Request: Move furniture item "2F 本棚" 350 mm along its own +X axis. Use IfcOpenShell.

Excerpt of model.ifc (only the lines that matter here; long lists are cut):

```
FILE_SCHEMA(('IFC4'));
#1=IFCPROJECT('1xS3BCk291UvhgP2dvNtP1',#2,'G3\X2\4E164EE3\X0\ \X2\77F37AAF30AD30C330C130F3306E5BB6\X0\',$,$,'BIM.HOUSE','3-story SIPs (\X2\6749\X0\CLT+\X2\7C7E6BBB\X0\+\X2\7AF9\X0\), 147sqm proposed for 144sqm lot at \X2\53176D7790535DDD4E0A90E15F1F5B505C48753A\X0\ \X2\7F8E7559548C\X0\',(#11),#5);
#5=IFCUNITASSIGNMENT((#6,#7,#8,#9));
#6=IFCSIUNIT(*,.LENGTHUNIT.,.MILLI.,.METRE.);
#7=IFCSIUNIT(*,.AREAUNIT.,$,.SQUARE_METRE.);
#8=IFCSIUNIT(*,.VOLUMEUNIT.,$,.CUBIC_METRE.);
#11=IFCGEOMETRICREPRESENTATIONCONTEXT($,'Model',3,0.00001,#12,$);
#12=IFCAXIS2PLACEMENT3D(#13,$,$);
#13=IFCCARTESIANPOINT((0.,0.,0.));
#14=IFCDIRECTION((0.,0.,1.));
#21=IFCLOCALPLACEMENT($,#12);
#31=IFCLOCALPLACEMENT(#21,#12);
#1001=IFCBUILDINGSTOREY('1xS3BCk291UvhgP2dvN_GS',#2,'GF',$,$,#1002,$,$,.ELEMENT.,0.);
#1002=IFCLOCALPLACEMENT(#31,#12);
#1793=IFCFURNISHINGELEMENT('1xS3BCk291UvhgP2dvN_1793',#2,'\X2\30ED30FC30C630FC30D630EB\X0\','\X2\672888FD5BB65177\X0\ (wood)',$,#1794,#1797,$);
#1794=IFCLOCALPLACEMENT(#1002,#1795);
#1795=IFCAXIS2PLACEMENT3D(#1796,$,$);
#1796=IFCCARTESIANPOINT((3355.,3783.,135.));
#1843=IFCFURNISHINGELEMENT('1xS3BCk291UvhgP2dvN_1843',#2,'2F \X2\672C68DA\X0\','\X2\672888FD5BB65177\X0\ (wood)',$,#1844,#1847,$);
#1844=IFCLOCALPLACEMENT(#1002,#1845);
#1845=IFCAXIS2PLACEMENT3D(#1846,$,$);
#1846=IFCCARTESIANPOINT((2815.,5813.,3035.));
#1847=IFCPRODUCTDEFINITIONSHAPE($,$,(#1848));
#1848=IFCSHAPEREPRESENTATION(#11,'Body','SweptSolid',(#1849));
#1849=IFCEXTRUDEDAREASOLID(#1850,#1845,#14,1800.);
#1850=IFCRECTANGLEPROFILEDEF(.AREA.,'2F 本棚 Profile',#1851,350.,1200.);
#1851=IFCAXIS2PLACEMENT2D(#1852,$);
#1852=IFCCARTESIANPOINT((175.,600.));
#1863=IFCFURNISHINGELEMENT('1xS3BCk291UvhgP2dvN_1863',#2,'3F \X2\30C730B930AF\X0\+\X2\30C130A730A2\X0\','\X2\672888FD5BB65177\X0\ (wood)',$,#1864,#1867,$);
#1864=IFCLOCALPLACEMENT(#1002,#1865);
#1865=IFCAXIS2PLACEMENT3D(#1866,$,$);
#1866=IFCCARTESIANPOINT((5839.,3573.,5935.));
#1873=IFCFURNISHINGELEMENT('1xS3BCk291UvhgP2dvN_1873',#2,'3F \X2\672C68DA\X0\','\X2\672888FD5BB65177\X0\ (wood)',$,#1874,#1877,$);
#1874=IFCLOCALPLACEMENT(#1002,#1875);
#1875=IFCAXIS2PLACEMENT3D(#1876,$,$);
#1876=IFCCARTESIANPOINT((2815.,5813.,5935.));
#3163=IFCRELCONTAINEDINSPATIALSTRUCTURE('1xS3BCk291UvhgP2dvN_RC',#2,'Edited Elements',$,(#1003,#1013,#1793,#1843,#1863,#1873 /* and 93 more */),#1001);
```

```python
import ifcopenshell
import ifcopenshell.api.geometry
import ifcopenshell.util.placement

model = ifcopenshell.open("model.ifc")

item = model.by_guid("1xS3BCk291UvhgP2dvN_1843")
matrix = ifcopenshell.util.placement.get_local_placement(item.ObjectPlacement)
matrix[:3, 3] += matrix[:3, 0] * 350.0
ifcopenshell.api.geometry.edit_object_placement(model, product=item, matrix=matrix, is_si=False)

print(ifcopenshell.util.placement.get_local_placement(item.ObjectPlacement).round(3) + 0.0)

model.write("model_updated.ifc")
```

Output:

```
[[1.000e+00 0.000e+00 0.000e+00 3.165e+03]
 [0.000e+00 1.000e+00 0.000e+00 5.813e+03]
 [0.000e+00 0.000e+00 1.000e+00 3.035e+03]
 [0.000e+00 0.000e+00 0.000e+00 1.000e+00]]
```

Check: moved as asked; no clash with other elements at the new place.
